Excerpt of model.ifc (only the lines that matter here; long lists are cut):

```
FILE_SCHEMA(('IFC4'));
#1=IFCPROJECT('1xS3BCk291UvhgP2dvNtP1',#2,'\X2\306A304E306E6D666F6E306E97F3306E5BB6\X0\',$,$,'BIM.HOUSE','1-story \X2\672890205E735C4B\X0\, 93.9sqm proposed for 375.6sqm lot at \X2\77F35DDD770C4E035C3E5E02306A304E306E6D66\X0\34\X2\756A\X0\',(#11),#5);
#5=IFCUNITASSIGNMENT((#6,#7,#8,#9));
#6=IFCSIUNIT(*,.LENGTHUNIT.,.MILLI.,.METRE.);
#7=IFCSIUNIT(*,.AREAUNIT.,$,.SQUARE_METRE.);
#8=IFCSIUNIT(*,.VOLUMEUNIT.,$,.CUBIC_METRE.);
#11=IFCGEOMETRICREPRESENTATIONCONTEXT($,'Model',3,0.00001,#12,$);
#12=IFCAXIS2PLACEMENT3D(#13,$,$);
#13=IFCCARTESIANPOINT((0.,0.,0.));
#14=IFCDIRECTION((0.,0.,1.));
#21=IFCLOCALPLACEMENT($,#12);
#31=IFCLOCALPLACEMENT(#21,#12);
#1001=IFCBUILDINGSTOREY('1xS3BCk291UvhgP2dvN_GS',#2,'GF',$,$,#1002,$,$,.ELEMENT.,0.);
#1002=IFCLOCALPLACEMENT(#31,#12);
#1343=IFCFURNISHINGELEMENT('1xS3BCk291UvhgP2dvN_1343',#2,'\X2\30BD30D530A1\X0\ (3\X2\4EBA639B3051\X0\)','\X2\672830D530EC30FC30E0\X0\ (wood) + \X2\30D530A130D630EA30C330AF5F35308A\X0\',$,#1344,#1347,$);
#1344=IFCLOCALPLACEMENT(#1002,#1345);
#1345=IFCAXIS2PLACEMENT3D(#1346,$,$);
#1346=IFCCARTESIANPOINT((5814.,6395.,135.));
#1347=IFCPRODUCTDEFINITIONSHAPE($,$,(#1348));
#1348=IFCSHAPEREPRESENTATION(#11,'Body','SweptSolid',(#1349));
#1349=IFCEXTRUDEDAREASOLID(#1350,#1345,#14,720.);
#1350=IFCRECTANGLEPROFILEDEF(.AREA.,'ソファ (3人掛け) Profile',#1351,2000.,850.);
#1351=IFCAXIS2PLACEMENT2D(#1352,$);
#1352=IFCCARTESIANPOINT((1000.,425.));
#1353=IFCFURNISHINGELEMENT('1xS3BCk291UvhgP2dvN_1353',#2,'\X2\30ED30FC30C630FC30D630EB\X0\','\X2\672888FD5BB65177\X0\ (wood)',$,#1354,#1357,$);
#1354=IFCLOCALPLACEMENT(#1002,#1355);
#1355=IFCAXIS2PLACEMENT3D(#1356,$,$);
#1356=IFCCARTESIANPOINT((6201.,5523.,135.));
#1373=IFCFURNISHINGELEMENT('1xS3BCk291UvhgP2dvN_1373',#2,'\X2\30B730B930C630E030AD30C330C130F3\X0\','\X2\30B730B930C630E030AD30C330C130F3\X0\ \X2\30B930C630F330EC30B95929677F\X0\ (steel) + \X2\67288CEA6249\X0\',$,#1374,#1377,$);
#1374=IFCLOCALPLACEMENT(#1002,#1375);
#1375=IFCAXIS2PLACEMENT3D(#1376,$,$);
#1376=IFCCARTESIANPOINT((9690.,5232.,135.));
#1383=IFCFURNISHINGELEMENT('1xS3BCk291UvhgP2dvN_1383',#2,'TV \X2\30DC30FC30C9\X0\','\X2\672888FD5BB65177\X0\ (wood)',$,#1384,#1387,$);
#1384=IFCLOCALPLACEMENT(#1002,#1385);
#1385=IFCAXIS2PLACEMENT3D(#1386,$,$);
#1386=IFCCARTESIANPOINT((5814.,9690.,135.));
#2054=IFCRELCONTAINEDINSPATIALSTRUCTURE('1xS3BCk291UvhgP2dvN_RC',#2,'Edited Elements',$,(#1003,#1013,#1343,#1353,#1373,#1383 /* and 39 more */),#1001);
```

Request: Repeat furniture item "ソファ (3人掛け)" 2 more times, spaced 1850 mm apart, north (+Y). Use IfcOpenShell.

```python
import numpy as np
import ifcopenshell
import ifcopenshell.api.geometry
import ifcopenshell.api.root
import ifcopenshell.util.element
import ifcopenshell.util.placement
import ifcopenshell.util.unit

model = ifcopenshell.open("model.ifc")
unit_scale = ifcopenshell.util.unit.calculate_unit_scale(model)


def reuse_history(source, copy):
    """copy_class also copies each property set's owner history, people and application; keep the originals."""
    for rel in copy.IsDefinedBy:
        if rel.is_a("IfcRelDefinesByProperties") and (history := rel.RelatingPropertyDefinition.OwnerHistory):
            rel.RelatingPropertyDefinition.OwnerHistory = source.OwnerHistory
            ifcopenshell.util.element.remove_deep2(model, history)


source = model.by_guid("1xS3BCk291UvhgP2dvN_1343")
base = ifcopenshell.util.placement.get_local_placement(source.ObjectPlacement)
step = np.array([0.0, 1.0, 0.0]) * 1.85 / unit_scale

for i in range(1, 3):
    copy = ifcopenshell.api.root.copy_class(model, product=source)
    copy.Representation = ifcopenshell.util.element.copy_deep(
        model, source.Representation, exclude=["IfcGeometricRepresentationContext", "IfcRepresentationMap"]
    )
    reuse_history(source, copy)
    matrix = base.copy()
    matrix[:3, 3] += i * step
    print("added at", matrix[:3, 3].round(3) + 0.0)
    ifcopenshell.api.geometry.edit_object_placement(model, product=copy, matrix=matrix, is_si=False)

model.write("model_rev.ifc")
```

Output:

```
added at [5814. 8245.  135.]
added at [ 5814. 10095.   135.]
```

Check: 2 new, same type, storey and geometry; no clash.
